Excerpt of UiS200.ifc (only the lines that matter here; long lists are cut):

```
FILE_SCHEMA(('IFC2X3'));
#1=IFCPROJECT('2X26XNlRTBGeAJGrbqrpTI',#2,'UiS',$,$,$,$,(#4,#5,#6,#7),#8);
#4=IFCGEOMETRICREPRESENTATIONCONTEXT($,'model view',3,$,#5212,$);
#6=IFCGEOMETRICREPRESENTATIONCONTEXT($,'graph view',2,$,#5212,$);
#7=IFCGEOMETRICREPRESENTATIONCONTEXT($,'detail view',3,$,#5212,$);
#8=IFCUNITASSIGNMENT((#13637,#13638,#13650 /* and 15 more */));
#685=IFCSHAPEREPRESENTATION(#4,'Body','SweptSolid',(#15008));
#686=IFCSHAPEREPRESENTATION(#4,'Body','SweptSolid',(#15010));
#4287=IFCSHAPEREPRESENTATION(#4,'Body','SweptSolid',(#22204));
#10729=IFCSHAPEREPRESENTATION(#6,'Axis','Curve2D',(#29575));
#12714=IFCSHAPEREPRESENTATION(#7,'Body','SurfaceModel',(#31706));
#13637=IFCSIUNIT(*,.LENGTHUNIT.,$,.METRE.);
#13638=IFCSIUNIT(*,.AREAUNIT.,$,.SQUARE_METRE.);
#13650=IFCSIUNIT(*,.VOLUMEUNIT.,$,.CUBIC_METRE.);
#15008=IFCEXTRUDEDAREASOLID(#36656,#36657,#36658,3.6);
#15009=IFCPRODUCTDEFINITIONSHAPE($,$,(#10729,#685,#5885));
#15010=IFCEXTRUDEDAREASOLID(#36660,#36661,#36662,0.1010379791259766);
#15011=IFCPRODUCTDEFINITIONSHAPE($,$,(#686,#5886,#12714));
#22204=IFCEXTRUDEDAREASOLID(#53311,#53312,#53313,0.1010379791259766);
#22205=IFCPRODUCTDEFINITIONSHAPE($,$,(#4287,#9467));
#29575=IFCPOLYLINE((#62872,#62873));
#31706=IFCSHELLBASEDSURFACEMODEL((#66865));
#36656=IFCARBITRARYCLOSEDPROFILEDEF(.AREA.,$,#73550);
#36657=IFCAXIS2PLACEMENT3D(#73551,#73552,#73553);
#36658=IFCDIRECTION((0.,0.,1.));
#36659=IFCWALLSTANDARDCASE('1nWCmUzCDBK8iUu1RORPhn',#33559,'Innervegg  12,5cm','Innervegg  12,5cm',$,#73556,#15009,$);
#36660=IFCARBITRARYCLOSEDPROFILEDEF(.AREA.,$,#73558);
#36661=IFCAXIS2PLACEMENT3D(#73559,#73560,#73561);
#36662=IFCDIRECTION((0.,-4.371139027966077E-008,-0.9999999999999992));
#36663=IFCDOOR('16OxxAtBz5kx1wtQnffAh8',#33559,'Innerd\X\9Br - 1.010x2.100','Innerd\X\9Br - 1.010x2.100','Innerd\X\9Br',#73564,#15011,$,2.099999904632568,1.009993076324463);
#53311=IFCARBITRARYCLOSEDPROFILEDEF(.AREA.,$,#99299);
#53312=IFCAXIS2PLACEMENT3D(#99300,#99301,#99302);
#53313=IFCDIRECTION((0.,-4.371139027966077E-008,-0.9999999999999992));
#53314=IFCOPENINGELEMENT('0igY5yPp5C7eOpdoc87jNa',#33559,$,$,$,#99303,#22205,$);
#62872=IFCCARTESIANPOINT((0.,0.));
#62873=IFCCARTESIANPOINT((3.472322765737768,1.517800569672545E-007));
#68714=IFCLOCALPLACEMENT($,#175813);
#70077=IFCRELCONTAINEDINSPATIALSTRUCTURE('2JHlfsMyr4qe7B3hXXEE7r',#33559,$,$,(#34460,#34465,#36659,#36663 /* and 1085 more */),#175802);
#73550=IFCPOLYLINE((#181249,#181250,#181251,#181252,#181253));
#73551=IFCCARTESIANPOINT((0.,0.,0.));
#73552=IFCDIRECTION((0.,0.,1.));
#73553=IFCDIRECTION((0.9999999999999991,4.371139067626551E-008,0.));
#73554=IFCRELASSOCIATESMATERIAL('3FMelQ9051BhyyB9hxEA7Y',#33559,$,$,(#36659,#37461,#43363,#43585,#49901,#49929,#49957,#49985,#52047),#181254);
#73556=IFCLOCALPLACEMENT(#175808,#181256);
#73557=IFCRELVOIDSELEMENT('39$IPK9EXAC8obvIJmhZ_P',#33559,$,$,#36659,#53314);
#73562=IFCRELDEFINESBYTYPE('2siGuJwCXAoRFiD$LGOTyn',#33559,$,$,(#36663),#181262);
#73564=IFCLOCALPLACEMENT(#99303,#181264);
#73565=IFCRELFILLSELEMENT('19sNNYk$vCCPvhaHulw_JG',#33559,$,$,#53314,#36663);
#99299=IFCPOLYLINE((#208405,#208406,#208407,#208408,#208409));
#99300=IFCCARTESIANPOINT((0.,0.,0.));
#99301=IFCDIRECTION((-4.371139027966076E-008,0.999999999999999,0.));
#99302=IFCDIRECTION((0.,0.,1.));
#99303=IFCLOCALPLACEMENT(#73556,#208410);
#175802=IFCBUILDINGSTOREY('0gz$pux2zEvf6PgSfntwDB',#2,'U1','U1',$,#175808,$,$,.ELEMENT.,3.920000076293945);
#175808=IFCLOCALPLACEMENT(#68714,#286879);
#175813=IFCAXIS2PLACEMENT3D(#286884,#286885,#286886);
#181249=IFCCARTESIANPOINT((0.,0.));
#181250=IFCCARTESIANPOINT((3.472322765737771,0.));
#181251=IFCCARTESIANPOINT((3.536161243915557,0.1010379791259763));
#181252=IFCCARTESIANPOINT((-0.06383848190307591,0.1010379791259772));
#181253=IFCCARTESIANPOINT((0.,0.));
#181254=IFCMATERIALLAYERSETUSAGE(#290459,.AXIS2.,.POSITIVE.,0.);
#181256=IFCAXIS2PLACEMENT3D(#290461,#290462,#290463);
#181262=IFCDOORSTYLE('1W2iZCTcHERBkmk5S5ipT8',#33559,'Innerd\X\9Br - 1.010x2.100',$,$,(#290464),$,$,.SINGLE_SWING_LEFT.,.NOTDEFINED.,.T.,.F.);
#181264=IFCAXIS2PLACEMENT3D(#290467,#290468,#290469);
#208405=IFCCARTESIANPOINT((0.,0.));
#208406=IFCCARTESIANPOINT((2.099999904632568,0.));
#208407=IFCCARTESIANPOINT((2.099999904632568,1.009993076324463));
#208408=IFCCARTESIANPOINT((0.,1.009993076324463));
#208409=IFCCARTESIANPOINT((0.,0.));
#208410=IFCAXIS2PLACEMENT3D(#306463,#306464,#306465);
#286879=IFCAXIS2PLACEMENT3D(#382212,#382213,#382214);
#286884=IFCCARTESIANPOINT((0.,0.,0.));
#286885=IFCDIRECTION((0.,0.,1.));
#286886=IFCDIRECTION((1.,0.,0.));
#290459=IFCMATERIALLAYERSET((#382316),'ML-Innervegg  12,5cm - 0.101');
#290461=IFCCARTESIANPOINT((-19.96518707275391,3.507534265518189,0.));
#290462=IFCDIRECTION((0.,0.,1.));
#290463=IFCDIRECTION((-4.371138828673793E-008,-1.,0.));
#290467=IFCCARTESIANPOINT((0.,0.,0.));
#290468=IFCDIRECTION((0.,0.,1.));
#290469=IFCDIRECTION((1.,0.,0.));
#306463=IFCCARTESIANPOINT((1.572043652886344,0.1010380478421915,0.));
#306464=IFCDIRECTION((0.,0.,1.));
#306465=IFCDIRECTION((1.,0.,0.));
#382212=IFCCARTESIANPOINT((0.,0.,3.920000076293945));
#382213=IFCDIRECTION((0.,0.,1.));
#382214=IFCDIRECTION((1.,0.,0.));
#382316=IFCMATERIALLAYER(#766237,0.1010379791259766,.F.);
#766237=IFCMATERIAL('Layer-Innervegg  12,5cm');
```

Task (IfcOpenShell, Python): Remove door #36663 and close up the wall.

```python
import ifcopenshell
import ifcopenshell.api.feature
import ifcopenshell.api.root
import ifcopenshell.geom
import ifcopenshell.util.shape

model = ifcopenshell.open("UiS200.ifc")
settings = ifcopenshell.geom.settings()


def volume(element):
    """Net volume in cubic metres, openings subtracted."""
    shape = ifcopenshell.geom.create_shape(settings, element)
    return ifcopenshell.util.shape.get_volume(shape.geometry)


door = model.by_guid("16OxxAtBz5kx1wtQnffAh8")
opening = door.FillsVoids[0].RelatingOpeningElement
wall = opening.VoidsElements[0].RelatingBuildingElement
before = volume(wall)

ifcopenshell.api.root.remove_product(model, product=door)
ifcopenshell.api.feature.remove_feature(model, feature=opening)

after = volume(wall)

print(f"wall volume {before:.3f} -> {after:.3f} m3")

model.write("UiS200-out.ifc")
```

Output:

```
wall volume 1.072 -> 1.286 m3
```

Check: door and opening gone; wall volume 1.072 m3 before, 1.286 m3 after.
